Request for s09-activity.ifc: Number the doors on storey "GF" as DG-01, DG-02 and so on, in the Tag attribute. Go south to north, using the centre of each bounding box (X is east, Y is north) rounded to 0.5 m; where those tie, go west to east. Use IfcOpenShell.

First a look at what the model holds.

```python
import ifcopenshell
import ifcopenshell.util.element
import ifcopenshell.util.placement

model = ifcopenshell.open("s09-activity.ifc")
print(model.schema)
storey = next(s for s in model.by_type("IfcBuildingStorey") if s.Name == "GF")
doors = [e for e in ifcopenshell.util.element.get_decomposition(storey) if e.is_a("IfcDoor")]
for e in sorted(doors, key=lambda e: e.id()):
    origin = ifcopenshell.util.placement.get_local_placement(e.ObjectPlacement)[:3, 3]
    print(e.id(), e.Tag, e.Name, origin.round(2) + 0.0, sep=" | ")
```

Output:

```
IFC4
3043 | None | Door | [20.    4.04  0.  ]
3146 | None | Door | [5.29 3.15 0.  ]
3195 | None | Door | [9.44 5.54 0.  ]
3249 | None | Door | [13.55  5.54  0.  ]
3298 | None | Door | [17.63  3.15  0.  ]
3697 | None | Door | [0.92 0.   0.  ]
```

```python
import ifcopenshell
import ifcopenshell.geom
import ifcopenshell.util.element
import ifcopenshell.util.shape

model = ifcopenshell.open("s09-activity.ifc")
settings = ifcopenshell.geom.settings()
settings.set("use-world-coords", True)


def centre(element):
    shape = ifcopenshell.geom.create_shape(settings, element)
    return ifcopenshell.util.shape.get_bbox_centroid(shape.geometry)


storey = next(s for s in model.by_type("IfcBuildingStorey") if s.Name == "GF")
doors = [e for e in ifcopenshell.util.element.get_decomposition(storey) if e.is_a("IfcDoor")]

# Insertion points can sit at a corner or the storey origin, so sort by the geometry (in metres).
centres = {e: centre(e) for e in doors}
doors.sort(key=lambda e: (round(centres[e][1] / 0.5), centres[e][0]))

for i, e in enumerate(doors, start=1):
    number = f"DG-{i:02d}"
    e.Tag = number
    print(e.id(), number)

model.write("s09-activity_v2.ifc")
```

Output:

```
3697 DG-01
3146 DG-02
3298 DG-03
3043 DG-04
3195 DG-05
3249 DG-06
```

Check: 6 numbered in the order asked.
